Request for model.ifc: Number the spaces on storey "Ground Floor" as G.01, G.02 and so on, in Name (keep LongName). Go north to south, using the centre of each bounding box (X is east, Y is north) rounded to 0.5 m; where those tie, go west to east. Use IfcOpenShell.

First a look at what the model holds.

```python
import ifcopenshell
import ifcopenshell.util.element
import ifcopenshell.util.placement

model = ifcopenshell.open("model.ifc")
print(model.schema)
storey = next(s for s in model.by_type("IfcBuildingStorey") if s.Name == "Ground Floor")
spaces = [e for e in ifcopenshell.util.element.get_decomposition(storey) if e.is_a("IfcSpace")]
for e in sorted(spaces, key=lambda e: e.id()):
    origin = ifcopenshell.util.placement.get_local_placement(e.ObjectPlacement)[:3, 3]
    print(e.id(), e.Name, e.LongName, origin.round(2) + 0.0, sep=" | ")
```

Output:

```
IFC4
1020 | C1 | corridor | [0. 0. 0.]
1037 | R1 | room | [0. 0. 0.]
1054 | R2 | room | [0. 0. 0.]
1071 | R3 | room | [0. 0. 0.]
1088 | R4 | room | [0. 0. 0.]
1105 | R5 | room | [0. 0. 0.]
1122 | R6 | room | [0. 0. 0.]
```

```python
import ifcopenshell
import ifcopenshell.geom
import ifcopenshell.util.element
import ifcopenshell.util.shape

model = ifcopenshell.open("model.ifc")
settings = ifcopenshell.geom.settings()
settings.set("use-world-coords", True)


def centre(element):
    shape = ifcopenshell.geom.create_shape(settings, element)
    return ifcopenshell.util.shape.get_bbox_centroid(shape.geometry)


storey = next(s for s in model.by_type("IfcBuildingStorey") if s.Name == "Ground Floor")
spaces = [e for e in ifcopenshell.util.element.get_decomposition(storey) if e.is_a("IfcSpace")]

# Insertion points can sit at a corner or the storey origin, so sort by the geometry (in metres).
centres = {e: centre(e) for e in spaces}
spaces.sort(key=lambda e: (-round(centres[e][1] / 0.5), centres[e][0]))

for i, e in enumerate(spaces, start=1):
    number = f"G.{i:02d}"
    e.Name = number
    print(e.id(), number)

model.write("model_rev.ifc")
```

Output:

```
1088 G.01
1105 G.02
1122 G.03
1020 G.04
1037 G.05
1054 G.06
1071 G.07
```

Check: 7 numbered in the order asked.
